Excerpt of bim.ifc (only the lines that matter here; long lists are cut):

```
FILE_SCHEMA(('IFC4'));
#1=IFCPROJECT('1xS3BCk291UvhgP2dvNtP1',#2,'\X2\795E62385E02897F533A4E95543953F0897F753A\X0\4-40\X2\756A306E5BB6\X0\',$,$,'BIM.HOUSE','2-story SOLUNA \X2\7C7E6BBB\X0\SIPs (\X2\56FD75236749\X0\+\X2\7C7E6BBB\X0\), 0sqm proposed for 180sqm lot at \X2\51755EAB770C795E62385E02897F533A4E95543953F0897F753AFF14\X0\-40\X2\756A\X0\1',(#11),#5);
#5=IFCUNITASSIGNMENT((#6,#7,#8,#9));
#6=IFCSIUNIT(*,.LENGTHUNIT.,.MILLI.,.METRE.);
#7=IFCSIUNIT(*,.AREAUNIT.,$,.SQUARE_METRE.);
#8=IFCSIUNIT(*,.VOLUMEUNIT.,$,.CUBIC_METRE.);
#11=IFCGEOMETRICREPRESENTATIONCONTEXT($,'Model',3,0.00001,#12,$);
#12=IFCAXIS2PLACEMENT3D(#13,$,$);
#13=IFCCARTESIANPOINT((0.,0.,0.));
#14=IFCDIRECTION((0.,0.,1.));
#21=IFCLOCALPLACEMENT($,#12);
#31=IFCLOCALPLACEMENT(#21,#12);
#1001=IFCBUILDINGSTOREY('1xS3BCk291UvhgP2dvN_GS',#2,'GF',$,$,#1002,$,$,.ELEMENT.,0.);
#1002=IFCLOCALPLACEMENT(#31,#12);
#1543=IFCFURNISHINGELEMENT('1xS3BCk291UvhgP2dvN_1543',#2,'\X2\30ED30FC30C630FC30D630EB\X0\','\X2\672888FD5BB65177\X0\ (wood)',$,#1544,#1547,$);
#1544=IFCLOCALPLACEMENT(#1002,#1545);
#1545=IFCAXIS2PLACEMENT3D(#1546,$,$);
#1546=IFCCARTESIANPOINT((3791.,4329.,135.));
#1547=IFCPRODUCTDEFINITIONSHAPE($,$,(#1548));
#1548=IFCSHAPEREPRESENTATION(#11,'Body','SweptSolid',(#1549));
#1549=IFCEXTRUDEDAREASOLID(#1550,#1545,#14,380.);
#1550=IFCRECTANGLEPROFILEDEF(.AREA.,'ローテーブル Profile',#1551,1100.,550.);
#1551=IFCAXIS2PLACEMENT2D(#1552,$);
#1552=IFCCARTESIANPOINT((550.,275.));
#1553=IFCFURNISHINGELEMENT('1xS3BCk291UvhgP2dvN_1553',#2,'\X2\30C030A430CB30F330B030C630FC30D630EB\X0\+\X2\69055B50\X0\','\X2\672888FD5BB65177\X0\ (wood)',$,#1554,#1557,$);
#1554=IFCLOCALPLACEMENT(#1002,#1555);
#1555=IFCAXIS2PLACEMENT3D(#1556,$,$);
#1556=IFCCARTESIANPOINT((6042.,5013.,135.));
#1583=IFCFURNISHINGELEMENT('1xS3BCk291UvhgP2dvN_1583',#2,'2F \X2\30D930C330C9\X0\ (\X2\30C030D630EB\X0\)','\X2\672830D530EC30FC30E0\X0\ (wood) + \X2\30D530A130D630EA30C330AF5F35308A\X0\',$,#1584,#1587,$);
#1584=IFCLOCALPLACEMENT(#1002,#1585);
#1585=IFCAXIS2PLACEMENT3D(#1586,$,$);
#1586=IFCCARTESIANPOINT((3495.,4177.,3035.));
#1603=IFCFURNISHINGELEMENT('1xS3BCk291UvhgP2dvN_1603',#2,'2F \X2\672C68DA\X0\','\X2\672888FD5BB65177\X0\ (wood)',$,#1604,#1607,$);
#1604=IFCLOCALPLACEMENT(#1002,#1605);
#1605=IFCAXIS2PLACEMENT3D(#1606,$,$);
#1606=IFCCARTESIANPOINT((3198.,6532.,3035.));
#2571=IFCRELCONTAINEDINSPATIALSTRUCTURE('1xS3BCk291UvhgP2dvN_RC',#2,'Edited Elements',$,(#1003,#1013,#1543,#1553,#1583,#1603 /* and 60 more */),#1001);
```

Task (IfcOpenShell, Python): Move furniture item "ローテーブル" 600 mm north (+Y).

```python
import ifcopenshell
import ifcopenshell.api.geometry
import ifcopenshell.util.placement
import ifcopenshell.util.unit

model = ifcopenshell.open("bim.ifc")
unit_scale = ifcopenshell.util.unit.calculate_unit_scale(model)

item = model.by_id(1543)
matrix = ifcopenshell.util.placement.get_local_placement(item.ObjectPlacement)
matrix[1, 3] += 0.6 / unit_scale
ifcopenshell.api.geometry.edit_object_placement(model, product=item, matrix=matrix, is_si=False)

print(ifcopenshell.util.placement.get_local_placement(item.ObjectPlacement).round(3) + 0.0)

model.write("bim_rev.ifc")
```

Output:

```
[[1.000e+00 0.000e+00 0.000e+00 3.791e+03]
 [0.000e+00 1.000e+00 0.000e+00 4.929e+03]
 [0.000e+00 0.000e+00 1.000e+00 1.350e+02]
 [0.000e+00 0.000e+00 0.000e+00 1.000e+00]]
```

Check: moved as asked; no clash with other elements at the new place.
